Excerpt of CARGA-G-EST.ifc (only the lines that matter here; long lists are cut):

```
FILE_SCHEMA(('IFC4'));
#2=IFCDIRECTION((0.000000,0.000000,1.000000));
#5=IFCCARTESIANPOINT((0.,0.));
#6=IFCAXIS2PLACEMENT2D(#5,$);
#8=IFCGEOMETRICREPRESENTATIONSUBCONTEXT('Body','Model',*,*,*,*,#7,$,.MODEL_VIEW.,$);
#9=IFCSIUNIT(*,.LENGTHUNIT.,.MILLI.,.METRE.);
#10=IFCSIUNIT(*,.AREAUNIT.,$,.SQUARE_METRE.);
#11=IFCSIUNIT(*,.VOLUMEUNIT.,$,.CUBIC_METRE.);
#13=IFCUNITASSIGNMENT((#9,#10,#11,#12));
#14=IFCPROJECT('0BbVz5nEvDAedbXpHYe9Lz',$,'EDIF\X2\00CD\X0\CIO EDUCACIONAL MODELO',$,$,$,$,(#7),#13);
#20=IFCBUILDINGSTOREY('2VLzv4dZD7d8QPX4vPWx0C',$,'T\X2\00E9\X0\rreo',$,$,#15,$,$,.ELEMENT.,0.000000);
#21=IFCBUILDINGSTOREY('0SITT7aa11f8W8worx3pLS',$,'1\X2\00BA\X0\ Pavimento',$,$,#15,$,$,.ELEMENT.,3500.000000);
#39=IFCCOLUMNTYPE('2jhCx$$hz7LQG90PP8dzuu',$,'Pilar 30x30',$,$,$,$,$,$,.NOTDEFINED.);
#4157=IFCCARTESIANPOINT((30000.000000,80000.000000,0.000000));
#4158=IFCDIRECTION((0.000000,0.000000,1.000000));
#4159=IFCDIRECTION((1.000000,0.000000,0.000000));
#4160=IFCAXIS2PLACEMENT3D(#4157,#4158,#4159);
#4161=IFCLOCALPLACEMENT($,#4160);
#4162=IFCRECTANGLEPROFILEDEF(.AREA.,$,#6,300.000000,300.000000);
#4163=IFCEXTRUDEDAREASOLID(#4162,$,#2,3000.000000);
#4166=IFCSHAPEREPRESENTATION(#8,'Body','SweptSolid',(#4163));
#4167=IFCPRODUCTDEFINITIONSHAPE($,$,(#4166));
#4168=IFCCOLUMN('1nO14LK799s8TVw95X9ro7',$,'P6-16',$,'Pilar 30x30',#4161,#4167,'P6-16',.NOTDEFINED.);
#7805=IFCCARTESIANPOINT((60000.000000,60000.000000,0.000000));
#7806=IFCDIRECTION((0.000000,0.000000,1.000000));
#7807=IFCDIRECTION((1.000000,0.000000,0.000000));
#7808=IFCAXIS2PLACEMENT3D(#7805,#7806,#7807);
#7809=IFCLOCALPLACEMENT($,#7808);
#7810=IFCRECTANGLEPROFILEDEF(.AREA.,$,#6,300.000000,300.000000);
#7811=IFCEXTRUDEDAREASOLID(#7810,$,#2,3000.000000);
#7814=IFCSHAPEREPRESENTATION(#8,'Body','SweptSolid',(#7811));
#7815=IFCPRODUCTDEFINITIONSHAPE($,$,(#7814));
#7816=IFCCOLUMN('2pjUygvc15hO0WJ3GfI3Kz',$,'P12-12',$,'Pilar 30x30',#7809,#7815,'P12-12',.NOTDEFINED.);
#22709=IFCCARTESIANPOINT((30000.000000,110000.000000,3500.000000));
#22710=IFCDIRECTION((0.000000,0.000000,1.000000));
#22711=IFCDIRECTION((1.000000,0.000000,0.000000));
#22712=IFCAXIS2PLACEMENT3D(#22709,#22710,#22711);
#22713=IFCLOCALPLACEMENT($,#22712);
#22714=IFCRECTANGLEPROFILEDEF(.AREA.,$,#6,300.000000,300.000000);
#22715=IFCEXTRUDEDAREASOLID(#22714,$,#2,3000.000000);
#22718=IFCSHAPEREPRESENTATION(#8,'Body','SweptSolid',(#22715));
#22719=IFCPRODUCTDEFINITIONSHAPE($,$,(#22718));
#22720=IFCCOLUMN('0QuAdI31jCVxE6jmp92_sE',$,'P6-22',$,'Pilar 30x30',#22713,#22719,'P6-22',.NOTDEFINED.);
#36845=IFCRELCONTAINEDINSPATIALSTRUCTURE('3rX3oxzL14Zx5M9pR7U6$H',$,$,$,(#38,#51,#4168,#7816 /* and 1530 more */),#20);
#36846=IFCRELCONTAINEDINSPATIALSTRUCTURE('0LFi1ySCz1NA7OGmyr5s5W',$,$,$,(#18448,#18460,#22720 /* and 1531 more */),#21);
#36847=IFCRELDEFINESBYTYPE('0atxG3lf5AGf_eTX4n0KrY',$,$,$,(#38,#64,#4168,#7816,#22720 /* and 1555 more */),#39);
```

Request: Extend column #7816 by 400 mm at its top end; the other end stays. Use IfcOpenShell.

```python
import ifcopenshell
import ifcopenshell.util.representation

model = ifcopenshell.open("CARGA-G-EST.ifc")

member = model.by_guid("2pjUygvc15hO0WJ3GfI3Kz")
change = 400.0

# The extrusion runs towards the end named, so only its depth changes.
body = ifcopenshell.util.representation.get_representation(member, "Model", "Body")
solid = body.Items[0]
old_length = solid.Depth
solid.Depth += change

print(f"length {old_length:g} -> {solid.Depth:g}")

model.write("CARGA-G-EST-out.ifc")
```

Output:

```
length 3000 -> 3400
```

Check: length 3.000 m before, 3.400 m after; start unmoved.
